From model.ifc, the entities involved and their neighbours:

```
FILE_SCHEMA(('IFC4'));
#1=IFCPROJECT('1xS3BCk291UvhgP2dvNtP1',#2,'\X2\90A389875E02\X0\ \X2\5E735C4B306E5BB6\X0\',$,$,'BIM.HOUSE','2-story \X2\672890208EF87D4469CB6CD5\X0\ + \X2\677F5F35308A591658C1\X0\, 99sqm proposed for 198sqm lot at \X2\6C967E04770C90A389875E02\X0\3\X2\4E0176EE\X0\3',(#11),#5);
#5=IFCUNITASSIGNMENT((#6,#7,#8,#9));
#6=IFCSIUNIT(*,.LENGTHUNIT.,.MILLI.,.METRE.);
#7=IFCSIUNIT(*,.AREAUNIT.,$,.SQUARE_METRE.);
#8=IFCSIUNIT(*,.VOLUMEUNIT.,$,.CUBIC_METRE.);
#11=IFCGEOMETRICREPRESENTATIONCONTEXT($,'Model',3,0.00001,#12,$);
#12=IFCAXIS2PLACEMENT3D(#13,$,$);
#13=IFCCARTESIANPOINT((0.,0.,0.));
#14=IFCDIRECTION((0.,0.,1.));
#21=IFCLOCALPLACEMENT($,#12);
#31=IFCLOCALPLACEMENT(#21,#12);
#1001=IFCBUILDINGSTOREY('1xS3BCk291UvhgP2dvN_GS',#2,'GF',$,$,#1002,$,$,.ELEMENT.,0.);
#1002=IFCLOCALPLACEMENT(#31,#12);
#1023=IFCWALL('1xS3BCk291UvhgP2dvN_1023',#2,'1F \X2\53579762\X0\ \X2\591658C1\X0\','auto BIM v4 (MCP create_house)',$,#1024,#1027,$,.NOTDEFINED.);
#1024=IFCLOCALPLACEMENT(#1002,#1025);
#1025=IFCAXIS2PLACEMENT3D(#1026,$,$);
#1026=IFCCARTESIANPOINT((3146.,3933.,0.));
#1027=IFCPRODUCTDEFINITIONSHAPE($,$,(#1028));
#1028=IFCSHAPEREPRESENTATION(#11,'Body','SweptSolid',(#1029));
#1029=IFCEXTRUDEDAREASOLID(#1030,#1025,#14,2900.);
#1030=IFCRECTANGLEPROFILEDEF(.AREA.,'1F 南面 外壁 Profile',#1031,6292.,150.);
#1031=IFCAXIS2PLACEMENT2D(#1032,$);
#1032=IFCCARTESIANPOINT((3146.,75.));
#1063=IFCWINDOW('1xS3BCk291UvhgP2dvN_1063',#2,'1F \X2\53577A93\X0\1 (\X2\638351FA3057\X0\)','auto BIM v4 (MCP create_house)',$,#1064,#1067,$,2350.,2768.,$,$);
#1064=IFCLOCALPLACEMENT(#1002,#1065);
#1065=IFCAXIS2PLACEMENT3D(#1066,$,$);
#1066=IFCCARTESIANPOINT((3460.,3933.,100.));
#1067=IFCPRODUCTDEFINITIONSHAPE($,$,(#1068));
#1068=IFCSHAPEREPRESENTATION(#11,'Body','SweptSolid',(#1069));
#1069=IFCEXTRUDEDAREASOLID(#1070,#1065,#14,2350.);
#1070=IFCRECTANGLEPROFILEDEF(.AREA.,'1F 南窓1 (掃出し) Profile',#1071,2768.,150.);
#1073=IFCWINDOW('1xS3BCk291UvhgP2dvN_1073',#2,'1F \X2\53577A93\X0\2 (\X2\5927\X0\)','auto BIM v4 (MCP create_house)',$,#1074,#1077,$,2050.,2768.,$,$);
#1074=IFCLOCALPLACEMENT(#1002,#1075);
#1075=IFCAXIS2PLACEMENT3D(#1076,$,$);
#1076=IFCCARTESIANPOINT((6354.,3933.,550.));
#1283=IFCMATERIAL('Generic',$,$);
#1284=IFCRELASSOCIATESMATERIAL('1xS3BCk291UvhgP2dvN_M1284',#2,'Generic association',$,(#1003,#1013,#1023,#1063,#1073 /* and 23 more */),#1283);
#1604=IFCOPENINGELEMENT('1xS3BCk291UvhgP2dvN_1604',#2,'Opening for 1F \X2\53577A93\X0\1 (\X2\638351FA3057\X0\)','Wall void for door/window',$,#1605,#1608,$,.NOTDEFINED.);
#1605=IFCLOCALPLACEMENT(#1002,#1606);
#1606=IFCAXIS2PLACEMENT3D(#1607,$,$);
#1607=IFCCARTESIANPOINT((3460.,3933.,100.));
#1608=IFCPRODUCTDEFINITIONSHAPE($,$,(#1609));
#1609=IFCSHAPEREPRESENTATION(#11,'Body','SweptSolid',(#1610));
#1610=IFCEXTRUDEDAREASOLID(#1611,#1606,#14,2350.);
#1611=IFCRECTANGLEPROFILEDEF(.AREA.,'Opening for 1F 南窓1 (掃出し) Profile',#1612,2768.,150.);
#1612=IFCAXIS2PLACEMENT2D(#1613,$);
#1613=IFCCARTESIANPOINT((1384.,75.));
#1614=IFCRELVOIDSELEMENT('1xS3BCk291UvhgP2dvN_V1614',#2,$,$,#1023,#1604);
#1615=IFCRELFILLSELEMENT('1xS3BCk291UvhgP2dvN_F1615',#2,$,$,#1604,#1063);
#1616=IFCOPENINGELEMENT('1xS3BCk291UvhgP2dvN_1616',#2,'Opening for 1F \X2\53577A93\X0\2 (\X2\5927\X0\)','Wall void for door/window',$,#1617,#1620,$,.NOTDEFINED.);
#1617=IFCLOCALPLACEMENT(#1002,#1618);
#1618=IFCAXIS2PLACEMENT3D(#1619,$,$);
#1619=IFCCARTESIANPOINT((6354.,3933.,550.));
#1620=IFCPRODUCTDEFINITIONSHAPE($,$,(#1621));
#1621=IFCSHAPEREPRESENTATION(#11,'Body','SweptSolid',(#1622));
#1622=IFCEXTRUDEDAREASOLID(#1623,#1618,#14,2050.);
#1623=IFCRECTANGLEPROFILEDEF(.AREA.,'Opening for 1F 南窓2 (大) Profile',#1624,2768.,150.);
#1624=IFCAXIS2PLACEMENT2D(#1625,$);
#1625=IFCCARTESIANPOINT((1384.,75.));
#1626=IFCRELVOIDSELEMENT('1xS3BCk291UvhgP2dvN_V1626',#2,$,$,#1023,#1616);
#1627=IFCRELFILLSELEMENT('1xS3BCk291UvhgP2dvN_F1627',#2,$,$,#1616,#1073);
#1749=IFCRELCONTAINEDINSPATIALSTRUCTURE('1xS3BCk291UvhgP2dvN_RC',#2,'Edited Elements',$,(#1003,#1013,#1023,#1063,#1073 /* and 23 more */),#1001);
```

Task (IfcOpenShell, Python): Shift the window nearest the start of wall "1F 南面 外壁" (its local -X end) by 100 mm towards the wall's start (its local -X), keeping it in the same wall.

```python
import ifcopenshell
import ifcopenshell.api.geometry
import ifcopenshell.util.placement
import ifcopenshell.util.unit

model = ifcopenshell.open("model.ifc")
unit_scale = ifcopenshell.util.unit.calculate_unit_scale(model)

window = model.by_guid("1xS3BCk291UvhgP2dvN_1063")
opening = window.FillsVoids[0].RelatingOpeningElement
wall = opening.VoidsElements[0].RelatingBuildingElement

wall_matrix = ifcopenshell.util.placement.get_local_placement(wall.ObjectPlacement)
shift = wall_matrix[:3, 0] * -0.1 / unit_scale
before = ifcopenshell.util.placement.get_local_placement(window.ObjectPlacement)[:3, 3].copy()

# The window is not placed relative to its opening, so move both.
for product in (opening, window):
    matrix = ifcopenshell.util.placement.get_local_placement(product.ObjectPlacement)
    matrix[:3, 3] += shift
    ifcopenshell.api.geometry.edit_object_placement(model, product=product, matrix=matrix, is_si=False)

after = ifcopenshell.util.placement.get_local_placement(window.ObjectPlacement)[:3, 3]
print("window moved by", (after - before).round(3) + 0.0)

model.write("model-out.ifc")
```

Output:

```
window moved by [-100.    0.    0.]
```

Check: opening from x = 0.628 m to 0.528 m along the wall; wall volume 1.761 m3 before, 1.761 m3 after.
